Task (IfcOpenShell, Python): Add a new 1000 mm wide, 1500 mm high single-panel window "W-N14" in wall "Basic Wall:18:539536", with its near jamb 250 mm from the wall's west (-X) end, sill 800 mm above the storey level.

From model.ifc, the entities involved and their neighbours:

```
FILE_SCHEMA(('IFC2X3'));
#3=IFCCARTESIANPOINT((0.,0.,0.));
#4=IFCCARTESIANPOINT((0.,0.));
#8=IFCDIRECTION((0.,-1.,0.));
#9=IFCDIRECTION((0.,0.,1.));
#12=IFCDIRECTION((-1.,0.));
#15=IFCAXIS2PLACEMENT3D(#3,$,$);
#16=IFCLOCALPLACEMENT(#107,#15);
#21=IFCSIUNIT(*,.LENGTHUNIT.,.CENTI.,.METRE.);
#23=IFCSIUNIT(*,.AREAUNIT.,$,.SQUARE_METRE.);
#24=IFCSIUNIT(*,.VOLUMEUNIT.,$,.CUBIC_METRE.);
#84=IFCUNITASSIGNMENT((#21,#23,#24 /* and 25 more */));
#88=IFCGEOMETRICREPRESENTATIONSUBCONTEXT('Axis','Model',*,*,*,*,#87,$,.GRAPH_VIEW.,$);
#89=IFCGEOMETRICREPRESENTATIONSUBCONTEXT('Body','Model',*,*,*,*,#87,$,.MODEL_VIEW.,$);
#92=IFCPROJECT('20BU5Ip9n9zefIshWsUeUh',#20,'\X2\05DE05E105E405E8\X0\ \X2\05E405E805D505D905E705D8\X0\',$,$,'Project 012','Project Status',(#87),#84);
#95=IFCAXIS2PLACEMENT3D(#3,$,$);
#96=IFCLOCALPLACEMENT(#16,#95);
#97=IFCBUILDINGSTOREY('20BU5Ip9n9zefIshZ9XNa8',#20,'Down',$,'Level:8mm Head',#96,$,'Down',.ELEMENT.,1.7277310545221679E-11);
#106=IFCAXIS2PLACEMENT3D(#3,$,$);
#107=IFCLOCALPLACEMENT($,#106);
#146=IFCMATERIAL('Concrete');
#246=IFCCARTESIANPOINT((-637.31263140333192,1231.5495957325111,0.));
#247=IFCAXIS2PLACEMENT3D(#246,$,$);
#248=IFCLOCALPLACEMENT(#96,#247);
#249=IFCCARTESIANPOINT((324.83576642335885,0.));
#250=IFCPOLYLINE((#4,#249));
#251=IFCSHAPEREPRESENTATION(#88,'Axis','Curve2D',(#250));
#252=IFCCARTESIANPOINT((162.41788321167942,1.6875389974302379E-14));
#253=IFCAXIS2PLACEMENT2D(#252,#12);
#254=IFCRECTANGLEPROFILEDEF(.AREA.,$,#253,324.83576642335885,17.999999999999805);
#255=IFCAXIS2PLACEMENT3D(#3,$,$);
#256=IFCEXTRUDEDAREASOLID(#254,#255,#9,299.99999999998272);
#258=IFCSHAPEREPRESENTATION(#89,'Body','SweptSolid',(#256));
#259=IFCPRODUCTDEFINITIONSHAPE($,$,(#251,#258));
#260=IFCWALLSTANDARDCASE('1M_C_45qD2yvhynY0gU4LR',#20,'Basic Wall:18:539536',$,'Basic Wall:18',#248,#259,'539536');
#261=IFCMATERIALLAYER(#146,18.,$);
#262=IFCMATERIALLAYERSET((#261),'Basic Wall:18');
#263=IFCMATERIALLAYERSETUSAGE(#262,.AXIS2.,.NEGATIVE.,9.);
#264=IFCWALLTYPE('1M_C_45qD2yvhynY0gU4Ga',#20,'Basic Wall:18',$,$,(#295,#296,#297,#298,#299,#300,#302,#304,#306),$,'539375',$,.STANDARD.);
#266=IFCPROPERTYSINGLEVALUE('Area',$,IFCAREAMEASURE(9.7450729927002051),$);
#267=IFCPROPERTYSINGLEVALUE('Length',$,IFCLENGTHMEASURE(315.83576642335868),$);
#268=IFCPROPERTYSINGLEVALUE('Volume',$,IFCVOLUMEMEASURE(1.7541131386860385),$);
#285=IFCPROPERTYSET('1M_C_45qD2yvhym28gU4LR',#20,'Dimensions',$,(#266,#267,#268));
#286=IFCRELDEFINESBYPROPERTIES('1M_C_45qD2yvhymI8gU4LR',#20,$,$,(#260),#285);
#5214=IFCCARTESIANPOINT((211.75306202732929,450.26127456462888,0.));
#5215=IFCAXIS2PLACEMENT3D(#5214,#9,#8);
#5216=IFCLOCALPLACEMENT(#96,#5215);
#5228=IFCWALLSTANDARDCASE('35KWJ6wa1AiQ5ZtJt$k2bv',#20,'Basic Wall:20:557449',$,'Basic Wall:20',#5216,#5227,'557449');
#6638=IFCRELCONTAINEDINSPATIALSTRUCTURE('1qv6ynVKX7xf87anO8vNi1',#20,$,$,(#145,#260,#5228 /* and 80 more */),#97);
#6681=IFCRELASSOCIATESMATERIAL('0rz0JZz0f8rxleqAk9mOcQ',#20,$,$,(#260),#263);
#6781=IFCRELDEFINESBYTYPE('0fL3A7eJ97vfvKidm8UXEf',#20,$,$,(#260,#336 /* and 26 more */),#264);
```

```python
import numpy as np
import ifcopenshell
import ifcopenshell.api.feature
import ifcopenshell.api.geometry
import ifcopenshell.api.pset
import ifcopenshell.api.root
import ifcopenshell.api.spatial
import ifcopenshell.api.type
import ifcopenshell.geom
import ifcopenshell.util.element
import ifcopenshell.util.placement
import ifcopenshell.util.representation
import ifcopenshell.util.shape
import ifcopenshell.util.unit

model = ifcopenshell.open("model.ifc")
unit_scale = ifcopenshell.util.unit.calculate_unit_scale(model)
area_scale = ifcopenshell.util.unit.calculate_unit_scale(model, "AREAUNIT")
volume_scale = ifcopenshell.util.unit.calculate_unit_scale(model, "VOLUMEUNIT")
settings = ifcopenshell.geom.settings()


def volume(element):
    """Net volume in cubic metres, openings subtracted."""
    shape = ifcopenshell.geom.create_shape(settings, element)
    return ifcopenshell.util.shape.get_volume(shape.geometry)


wall = model.by_id(260)
storey = ifcopenshell.util.element.get_container(wall, ifc_class="IfcBuildingStorey")
context = ifcopenshell.util.representation.get_context(model, "Model", "Body", "MODEL_VIEW")
before = volume(wall)

width, height, from_end, sill = 1, 1.5, 0.25, 0.8  # metres

# The wall runs along its own X axis, and the end named is its -X end.
wall_shape = ifcopenshell.geom.create_shape(settings, wall)
x, y, z = ifcopenshell.util.shape.get_vertices(wall_shape.geometry).T
start = x.min() + from_end
face, thickness = float(y.min()), float(y.max() - y.min())
wall_matrix = ifcopenshell.util.placement.get_local_placement(wall.ObjectPlacement)
level = ifcopenshell.util.placement.get_local_placement(storey.ObjectPlacement)[2, 3]


def in_wall(x, y):
    """Placement at x, y metres in the wall's axes, at sill height."""
    matrix = wall_matrix.copy()
    matrix[:, 3] = wall_matrix @ np.array([x / unit_scale, y / unit_scale, 0.0, 1.0])
    matrix[2, 3] = level + sill / unit_scale
    return matrix


# Opening: a box that overshoots both wall faces by 50 mm.
opening = ifcopenshell.api.root.create_entity(model, ifc_class="IfcOpeningElement")
box = ifcopenshell.api.geometry.add_wall_representation(
    model, context=context, length=width, height=height, thickness=thickness + 0.1
)
ifcopenshell.api.geometry.assign_representation(model, product=opening, representation=box)
ifcopenshell.api.geometry.edit_object_placement(model, product=opening, matrix=in_wall(start, face - 0.05), is_si=False)
ifcopenshell.api.feature.add_feature(model, feature=opening, element=wall)

window = ifcopenshell.api.root.create_entity(model, ifc_class="IfcWindow", name="W-N14")
window.OverallWidth, window.OverallHeight = width / unit_scale, height / unit_scale
body = ifcopenshell.api.geometry.add_window_representation(
    model,
    context=context,
    overall_width=window.OverallWidth,
    overall_height=window.OverallHeight,
    partition_type="SINGLE_PANEL",
)
ifcopenshell.api.geometry.assign_representation(model, product=window, representation=body)
ifcopenshell.api.spatial.assign_container(model, products=[window], relating_structure=storey)
fills = ifcopenshell.api.feature.add_filling(model, opening=opening, element=window)
fills.OwnerHistory = window.OwnerHistory  # required in IFC2X3

# IFC2X3 keeps the operation on the window style.
style = ifcopenshell.api.root.create_entity(model, ifc_class="IfcWindowStyle", name="W-N14")
style.OperationType, style.ConstructionType = "SINGLE_PANEL", "NOTDEFINED"
style.ParameterTakesPrecedence = style.Sizeable = False
ifcopenshell.api.type.assign_type(model, related_objects=[window], relating_type=style)

# Centre the window in the wall's thickness.
ifcopenshell.api.geometry.edit_object_placement(model, product=window, matrix=in_wall(start, face), is_si=False)
window_shape = ifcopenshell.geom.create_shape(settings, window)
depth = ifcopenshell.util.shape.get_vertices(window_shape.geometry)[:, 1]
offset = face + thickness / 2 - (depth.min() + depth.max()) / 2
ifcopenshell.api.geometry.edit_object_placement(model, product=window, matrix=in_wall(start, offset), is_si=False)

after = volume(wall)

# Update the wall's stored quantities.
pset = model.by_id(ifcopenshell.util.element.get_pset(wall, "Dimensions", should_inherit=False)["id"])
ifcopenshell.api.pset.edit_pset(model, pset=pset, properties={
    "Area": model.create_entity("IfcAreaMeasure", after / thickness / area_scale),
    "Volume": model.create_entity("IfcVolumeMeasure", after / volume_scale),
})

print(f"wall volume {before:.3f} -> {after:.3f} m3")

model.write("model-out.ifc")
```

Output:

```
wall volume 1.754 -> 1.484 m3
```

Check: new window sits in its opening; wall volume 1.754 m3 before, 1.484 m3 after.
